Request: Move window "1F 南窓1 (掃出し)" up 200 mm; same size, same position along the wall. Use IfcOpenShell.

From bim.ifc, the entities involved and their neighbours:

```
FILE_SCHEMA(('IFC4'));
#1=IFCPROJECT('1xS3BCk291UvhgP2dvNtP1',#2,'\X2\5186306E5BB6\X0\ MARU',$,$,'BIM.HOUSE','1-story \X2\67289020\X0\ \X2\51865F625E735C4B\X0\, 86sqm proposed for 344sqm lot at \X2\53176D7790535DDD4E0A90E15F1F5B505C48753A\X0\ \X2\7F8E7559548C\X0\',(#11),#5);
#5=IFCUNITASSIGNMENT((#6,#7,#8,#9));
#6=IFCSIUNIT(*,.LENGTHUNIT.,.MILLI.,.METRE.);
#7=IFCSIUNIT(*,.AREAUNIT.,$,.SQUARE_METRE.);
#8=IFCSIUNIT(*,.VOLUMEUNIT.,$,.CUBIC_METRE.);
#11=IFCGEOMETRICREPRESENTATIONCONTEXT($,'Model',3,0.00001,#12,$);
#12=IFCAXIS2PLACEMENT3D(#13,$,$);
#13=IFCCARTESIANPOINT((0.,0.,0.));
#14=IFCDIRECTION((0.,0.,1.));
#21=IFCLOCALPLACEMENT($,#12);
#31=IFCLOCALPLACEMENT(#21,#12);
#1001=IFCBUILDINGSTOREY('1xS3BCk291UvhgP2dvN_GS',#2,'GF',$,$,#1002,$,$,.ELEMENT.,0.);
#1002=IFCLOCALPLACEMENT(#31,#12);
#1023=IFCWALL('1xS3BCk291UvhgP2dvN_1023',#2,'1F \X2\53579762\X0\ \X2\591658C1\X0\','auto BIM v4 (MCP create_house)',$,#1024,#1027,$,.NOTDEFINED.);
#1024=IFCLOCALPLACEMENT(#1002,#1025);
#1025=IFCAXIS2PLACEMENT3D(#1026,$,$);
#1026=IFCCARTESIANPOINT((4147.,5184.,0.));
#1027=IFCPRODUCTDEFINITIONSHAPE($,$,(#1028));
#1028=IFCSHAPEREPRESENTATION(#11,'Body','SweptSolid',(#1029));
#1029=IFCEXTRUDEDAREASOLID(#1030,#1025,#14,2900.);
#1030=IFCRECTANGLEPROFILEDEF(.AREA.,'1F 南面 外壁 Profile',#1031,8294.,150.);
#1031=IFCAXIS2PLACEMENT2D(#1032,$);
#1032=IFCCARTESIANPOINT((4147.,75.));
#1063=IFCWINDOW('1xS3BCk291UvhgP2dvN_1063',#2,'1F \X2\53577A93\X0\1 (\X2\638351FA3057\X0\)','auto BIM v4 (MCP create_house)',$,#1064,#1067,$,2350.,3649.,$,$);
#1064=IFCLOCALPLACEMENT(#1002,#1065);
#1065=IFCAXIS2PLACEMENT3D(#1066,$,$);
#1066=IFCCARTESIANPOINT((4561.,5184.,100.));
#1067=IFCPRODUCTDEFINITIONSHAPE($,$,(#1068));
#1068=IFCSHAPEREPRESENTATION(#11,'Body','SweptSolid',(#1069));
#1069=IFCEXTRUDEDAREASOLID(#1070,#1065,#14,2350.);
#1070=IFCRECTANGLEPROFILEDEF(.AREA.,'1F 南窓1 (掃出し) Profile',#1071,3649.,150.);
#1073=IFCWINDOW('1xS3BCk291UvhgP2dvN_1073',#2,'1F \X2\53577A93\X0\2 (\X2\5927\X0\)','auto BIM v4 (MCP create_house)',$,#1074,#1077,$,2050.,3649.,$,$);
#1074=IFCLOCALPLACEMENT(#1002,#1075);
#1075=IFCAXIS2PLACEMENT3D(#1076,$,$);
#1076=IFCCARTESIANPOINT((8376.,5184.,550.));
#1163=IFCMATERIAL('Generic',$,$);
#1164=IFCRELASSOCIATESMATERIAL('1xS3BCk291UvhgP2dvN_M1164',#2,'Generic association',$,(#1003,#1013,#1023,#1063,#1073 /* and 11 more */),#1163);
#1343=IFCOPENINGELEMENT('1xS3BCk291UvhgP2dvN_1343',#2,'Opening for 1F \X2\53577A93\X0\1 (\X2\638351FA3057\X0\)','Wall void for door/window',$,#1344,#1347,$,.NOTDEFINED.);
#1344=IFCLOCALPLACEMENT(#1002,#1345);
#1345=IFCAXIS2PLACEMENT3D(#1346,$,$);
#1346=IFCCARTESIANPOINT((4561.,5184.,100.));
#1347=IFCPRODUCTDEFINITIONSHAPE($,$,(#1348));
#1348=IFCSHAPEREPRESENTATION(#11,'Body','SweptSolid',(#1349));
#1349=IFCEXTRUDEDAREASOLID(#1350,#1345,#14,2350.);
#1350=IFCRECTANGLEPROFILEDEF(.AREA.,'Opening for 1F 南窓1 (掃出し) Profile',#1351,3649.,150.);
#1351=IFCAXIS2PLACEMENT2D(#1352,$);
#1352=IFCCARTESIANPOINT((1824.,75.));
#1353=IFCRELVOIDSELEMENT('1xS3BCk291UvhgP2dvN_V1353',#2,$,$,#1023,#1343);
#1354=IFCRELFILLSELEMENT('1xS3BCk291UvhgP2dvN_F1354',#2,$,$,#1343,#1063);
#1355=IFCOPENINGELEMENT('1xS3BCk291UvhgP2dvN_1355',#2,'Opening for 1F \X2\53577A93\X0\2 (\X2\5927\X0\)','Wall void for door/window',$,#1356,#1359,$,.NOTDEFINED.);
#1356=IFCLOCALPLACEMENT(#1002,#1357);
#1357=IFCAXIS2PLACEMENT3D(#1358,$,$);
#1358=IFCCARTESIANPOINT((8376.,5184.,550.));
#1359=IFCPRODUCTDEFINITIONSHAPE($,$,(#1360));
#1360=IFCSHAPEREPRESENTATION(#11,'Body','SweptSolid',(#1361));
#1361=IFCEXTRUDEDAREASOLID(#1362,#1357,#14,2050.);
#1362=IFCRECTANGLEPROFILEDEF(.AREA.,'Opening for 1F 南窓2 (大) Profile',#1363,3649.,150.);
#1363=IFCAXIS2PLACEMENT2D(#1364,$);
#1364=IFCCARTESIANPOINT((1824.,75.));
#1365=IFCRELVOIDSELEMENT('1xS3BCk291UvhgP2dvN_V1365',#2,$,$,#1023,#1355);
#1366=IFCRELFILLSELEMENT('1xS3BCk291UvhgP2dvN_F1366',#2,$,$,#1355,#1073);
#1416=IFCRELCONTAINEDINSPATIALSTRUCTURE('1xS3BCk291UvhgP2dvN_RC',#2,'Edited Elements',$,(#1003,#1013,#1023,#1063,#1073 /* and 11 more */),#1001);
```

```python
import numpy as np
import ifcopenshell
import ifcopenshell.api.geometry
import ifcopenshell.util.placement
import ifcopenshell.util.unit

model = ifcopenshell.open("bim.ifc")
unit_scale = ifcopenshell.util.unit.calculate_unit_scale(model)

window = model.by_guid("1xS3BCk291UvhgP2dvN_1063")
opening = window.FillsVoids[0].RelatingOpeningElement
dz = 200.0

shift = np.array([0.0, 0.0, dz])
# The window is not placed relative to its opening, so move both.
for product in (opening, window):
    matrix = ifcopenshell.util.placement.get_local_placement(product.ObjectPlacement)
    matrix[:3, 3] += shift
    ifcopenshell.api.geometry.edit_object_placement(model, product=product, matrix=matrix, is_si=False)

print(f"moved by {dz * unit_scale:+.3f} m")

model.write("bim_edited.ifc")
```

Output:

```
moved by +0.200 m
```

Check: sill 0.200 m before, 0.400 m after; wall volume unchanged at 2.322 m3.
